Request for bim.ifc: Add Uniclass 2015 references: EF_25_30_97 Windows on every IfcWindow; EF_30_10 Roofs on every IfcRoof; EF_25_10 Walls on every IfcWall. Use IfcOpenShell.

First a look at what the model holds.

```python
import ifcopenshell

model = ifcopenshell.open("bim.ifc")
print(model.schema)
print("classifications:", [c.Name for c in model.by_type("IfcClassification")])
for ifc_class in ("IfcDoor", "IfcRoof", "IfcStair", "IfcWall", "IfcWindow"):
    print(ifc_class, len(model.by_type(ifc_class)))
```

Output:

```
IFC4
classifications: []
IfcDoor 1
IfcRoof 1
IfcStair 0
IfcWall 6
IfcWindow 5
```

```python
import ifcopenshell
import ifcopenshell.api.classification

model = ifcopenshell.open("bim.ifc")

system = ifcopenshell.api.classification.add_classification(model, classification="Uniclass 2015")

codes = {
    "IfcWindow": ("EF_25_30_97", "Windows"),
    "IfcRoof": ("EF_30_10", "Roofs"),
    "IfcWall": ("EF_25_10", "Walls"),
}
for ifc_class, (code, name) in codes.items():
    products = model.by_type(ifc_class)
    ifcopenshell.api.classification.add_reference(
        model, products=products, classification=system, identification=code, name=name
    )
    print(code, len(products))

model.write("bim_edited.ifc")
```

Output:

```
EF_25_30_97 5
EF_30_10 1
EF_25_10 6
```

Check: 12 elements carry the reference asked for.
